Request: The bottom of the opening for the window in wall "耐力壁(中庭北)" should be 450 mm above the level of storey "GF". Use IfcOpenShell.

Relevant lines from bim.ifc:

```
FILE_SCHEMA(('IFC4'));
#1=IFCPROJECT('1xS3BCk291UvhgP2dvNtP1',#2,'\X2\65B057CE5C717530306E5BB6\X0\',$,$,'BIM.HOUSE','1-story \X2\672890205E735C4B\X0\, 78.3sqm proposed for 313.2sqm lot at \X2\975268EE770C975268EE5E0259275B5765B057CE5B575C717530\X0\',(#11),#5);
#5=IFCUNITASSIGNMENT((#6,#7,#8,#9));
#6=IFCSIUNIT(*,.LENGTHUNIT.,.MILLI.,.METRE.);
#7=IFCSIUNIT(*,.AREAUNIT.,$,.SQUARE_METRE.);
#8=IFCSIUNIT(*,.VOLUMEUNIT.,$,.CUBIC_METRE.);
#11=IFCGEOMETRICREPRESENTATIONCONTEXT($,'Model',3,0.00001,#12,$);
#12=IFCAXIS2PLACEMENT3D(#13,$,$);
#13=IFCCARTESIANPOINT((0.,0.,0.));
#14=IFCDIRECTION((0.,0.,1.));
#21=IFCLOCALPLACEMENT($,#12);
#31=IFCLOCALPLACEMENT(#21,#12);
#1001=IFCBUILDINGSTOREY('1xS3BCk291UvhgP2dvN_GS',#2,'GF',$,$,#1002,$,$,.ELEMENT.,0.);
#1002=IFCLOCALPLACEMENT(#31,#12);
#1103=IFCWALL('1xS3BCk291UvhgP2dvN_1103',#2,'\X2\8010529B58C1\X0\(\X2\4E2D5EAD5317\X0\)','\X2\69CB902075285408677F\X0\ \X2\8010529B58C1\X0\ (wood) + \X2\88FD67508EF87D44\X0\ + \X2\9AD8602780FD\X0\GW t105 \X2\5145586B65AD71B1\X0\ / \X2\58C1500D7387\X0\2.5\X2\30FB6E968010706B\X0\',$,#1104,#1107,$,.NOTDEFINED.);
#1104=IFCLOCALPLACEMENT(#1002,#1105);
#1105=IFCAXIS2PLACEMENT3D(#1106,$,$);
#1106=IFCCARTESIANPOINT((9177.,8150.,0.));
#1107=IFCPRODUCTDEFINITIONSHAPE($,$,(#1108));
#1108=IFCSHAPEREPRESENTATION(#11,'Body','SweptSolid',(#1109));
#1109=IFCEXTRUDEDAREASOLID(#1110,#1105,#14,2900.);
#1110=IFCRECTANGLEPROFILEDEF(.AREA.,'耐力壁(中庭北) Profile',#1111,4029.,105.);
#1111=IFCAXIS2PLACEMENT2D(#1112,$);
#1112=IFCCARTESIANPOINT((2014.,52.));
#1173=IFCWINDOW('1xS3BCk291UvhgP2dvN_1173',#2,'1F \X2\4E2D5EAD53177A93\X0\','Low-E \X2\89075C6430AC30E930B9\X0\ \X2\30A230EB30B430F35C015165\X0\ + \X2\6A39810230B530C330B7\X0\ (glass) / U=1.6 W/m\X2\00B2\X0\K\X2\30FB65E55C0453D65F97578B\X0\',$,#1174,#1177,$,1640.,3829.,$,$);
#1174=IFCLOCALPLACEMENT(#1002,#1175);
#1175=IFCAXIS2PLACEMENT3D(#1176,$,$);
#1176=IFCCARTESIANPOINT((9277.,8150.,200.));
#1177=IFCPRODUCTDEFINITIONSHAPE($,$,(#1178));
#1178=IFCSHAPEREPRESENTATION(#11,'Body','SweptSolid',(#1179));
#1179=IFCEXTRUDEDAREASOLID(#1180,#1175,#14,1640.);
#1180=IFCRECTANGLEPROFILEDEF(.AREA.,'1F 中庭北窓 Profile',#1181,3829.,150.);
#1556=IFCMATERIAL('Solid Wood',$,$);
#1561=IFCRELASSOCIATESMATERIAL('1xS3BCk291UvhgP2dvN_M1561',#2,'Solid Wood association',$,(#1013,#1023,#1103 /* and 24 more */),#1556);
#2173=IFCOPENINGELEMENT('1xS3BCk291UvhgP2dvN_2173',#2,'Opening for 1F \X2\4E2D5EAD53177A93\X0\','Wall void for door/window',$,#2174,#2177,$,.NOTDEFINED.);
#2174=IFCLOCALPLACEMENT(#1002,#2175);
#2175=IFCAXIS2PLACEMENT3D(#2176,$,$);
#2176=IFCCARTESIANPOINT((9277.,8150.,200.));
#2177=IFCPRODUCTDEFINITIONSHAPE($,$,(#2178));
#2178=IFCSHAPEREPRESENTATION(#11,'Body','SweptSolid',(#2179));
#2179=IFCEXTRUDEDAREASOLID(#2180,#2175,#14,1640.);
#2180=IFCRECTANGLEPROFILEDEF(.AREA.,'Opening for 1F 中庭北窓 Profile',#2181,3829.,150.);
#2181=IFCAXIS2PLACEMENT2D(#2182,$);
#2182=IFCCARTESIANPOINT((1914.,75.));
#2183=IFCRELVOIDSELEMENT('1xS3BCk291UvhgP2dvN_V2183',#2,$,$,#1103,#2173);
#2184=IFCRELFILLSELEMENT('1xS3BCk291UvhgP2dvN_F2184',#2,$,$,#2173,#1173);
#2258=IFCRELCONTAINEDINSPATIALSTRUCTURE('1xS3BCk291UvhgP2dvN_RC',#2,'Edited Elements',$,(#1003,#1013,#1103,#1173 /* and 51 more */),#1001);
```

```python
import numpy as np
import ifcopenshell
import ifcopenshell.api.geometry
import ifcopenshell.geom
import ifcopenshell.util.element
import ifcopenshell.util.placement
import ifcopenshell.util.shape
import ifcopenshell.util.unit

model = ifcopenshell.open("bim.ifc")
unit_scale = ifcopenshell.util.unit.calculate_unit_scale(model)

window = model.by_guid("1xS3BCk291UvhgP2dvN_1173")
opening = window.FillsVoids[0].RelatingOpeningElement
storey = ifcopenshell.util.element.get_container(window, ifc_class="IfcBuildingStorey")
level = ifcopenshell.util.placement.get_local_placement(storey.ObjectPlacement)[2, 3]

# The opening's origin need not be at the sill, so measure its lowest point.
shape = ifcopenshell.geom.create_shape(ifcopenshell.geom.settings(), opening)
bottom = ifcopenshell.util.shape.get_shape_bottom_elevation(shape, shape.geometry) / unit_scale
dz = level + 0.45 / unit_scale - bottom

shift = np.array([0.0, 0.0, dz])
# The window is not placed relative to its opening, so move both.
for product in (opening, window):
    matrix = ifcopenshell.util.placement.get_local_placement(product.ObjectPlacement)
    matrix[:3, 3] += shift
    ifcopenshell.api.geometry.edit_object_placement(model, product=product, matrix=matrix, is_si=False)

print(f"moved by {dz * unit_scale:+.3f} m")

model.write("bim_edited.ifc")
```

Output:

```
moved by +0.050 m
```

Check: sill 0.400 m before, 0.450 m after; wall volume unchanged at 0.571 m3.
